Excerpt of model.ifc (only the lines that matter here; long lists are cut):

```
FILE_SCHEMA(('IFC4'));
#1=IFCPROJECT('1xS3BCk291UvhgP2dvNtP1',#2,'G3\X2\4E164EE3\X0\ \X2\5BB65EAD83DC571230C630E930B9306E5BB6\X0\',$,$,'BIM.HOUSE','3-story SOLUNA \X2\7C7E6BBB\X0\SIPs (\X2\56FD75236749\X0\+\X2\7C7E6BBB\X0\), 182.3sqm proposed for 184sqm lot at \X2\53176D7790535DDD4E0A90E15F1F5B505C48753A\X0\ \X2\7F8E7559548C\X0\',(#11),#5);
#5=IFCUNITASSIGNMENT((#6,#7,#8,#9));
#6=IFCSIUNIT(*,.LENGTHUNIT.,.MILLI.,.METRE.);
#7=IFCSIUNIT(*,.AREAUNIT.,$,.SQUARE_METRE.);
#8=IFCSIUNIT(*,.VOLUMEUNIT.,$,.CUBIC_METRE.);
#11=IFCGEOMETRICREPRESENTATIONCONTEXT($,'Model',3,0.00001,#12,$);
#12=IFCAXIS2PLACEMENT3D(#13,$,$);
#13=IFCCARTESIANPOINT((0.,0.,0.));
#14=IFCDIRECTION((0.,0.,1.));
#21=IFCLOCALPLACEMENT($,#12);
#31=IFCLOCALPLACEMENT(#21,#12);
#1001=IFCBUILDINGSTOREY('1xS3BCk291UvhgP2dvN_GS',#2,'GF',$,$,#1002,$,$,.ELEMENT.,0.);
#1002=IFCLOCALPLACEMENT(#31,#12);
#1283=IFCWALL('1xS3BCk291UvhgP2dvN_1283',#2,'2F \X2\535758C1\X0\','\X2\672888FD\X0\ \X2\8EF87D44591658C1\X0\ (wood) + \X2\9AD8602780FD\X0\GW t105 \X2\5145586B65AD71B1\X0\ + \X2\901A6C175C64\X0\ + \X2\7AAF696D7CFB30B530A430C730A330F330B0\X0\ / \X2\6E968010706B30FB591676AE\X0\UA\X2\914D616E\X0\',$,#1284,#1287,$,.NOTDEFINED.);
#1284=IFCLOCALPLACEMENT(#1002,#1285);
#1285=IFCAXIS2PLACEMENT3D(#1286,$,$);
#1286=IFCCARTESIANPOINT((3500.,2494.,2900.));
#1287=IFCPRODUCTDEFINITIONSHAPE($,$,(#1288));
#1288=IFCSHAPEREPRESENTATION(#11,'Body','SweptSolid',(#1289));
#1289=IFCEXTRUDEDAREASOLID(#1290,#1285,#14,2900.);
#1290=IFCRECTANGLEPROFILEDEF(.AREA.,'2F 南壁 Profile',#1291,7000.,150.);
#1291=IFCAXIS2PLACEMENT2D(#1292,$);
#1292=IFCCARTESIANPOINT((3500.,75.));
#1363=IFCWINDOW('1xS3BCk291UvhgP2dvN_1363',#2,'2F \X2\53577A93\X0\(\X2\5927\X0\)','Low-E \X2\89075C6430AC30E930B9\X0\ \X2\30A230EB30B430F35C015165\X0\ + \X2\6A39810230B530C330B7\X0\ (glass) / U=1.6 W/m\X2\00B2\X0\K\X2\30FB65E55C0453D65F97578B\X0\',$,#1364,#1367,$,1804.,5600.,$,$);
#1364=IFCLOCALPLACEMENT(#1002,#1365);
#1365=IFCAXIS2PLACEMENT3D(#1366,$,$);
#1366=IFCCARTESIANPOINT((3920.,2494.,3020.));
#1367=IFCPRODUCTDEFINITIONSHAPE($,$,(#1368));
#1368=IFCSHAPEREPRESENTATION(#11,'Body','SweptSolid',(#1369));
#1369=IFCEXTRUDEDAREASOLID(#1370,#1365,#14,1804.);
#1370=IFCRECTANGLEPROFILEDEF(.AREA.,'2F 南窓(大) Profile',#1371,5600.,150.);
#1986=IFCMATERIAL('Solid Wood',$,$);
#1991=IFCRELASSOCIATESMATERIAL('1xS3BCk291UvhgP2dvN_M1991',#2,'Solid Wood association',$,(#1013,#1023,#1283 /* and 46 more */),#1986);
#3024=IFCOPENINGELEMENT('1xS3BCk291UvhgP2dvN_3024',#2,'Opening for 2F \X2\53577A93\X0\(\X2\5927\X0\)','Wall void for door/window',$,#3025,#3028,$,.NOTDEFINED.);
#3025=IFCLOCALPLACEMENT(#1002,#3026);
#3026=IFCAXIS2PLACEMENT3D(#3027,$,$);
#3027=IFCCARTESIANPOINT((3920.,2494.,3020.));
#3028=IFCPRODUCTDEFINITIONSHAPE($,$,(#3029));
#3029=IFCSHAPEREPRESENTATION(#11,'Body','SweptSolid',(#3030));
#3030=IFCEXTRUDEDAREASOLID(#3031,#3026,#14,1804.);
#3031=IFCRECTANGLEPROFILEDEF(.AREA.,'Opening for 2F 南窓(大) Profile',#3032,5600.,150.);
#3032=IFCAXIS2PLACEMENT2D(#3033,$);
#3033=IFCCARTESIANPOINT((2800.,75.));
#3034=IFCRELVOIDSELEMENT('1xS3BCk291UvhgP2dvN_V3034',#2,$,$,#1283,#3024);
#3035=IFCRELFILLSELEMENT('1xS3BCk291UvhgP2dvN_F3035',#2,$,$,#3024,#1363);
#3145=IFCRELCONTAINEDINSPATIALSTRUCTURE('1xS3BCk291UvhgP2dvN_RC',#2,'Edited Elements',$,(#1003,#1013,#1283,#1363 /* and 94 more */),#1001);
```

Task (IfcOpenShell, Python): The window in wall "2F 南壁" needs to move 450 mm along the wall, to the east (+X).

```python
import ifcopenshell
import ifcopenshell.api.geometry
import ifcopenshell.util.placement

model = ifcopenshell.open("model.ifc")

window = model.by_guid("1xS3BCk291UvhgP2dvN_1363")
opening = window.FillsVoids[0].RelatingOpeningElement
wall = opening.VoidsElements[0].RelatingBuildingElement

wall_matrix = ifcopenshell.util.placement.get_local_placement(wall.ObjectPlacement)
shift = wall_matrix[:3, 0] * 450.0
before = ifcopenshell.util.placement.get_local_placement(window.ObjectPlacement)[:3, 3].copy()

# The window is not placed relative to its opening, so move both.
for product in (opening, window):
    matrix = ifcopenshell.util.placement.get_local_placement(product.ObjectPlacement)
    matrix[:3, 3] += shift
    ifcopenshell.api.geometry.edit_object_placement(model, product=product, matrix=matrix, is_si=False)

after = ifcopenshell.util.placement.get_local_placement(window.ObjectPlacement)[:3, 3]
print("window moved by", (after - before).round(3) + 0.0)

model.write("model-out.ifc")
```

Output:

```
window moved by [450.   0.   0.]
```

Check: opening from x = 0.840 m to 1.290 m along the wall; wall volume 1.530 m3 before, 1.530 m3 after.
